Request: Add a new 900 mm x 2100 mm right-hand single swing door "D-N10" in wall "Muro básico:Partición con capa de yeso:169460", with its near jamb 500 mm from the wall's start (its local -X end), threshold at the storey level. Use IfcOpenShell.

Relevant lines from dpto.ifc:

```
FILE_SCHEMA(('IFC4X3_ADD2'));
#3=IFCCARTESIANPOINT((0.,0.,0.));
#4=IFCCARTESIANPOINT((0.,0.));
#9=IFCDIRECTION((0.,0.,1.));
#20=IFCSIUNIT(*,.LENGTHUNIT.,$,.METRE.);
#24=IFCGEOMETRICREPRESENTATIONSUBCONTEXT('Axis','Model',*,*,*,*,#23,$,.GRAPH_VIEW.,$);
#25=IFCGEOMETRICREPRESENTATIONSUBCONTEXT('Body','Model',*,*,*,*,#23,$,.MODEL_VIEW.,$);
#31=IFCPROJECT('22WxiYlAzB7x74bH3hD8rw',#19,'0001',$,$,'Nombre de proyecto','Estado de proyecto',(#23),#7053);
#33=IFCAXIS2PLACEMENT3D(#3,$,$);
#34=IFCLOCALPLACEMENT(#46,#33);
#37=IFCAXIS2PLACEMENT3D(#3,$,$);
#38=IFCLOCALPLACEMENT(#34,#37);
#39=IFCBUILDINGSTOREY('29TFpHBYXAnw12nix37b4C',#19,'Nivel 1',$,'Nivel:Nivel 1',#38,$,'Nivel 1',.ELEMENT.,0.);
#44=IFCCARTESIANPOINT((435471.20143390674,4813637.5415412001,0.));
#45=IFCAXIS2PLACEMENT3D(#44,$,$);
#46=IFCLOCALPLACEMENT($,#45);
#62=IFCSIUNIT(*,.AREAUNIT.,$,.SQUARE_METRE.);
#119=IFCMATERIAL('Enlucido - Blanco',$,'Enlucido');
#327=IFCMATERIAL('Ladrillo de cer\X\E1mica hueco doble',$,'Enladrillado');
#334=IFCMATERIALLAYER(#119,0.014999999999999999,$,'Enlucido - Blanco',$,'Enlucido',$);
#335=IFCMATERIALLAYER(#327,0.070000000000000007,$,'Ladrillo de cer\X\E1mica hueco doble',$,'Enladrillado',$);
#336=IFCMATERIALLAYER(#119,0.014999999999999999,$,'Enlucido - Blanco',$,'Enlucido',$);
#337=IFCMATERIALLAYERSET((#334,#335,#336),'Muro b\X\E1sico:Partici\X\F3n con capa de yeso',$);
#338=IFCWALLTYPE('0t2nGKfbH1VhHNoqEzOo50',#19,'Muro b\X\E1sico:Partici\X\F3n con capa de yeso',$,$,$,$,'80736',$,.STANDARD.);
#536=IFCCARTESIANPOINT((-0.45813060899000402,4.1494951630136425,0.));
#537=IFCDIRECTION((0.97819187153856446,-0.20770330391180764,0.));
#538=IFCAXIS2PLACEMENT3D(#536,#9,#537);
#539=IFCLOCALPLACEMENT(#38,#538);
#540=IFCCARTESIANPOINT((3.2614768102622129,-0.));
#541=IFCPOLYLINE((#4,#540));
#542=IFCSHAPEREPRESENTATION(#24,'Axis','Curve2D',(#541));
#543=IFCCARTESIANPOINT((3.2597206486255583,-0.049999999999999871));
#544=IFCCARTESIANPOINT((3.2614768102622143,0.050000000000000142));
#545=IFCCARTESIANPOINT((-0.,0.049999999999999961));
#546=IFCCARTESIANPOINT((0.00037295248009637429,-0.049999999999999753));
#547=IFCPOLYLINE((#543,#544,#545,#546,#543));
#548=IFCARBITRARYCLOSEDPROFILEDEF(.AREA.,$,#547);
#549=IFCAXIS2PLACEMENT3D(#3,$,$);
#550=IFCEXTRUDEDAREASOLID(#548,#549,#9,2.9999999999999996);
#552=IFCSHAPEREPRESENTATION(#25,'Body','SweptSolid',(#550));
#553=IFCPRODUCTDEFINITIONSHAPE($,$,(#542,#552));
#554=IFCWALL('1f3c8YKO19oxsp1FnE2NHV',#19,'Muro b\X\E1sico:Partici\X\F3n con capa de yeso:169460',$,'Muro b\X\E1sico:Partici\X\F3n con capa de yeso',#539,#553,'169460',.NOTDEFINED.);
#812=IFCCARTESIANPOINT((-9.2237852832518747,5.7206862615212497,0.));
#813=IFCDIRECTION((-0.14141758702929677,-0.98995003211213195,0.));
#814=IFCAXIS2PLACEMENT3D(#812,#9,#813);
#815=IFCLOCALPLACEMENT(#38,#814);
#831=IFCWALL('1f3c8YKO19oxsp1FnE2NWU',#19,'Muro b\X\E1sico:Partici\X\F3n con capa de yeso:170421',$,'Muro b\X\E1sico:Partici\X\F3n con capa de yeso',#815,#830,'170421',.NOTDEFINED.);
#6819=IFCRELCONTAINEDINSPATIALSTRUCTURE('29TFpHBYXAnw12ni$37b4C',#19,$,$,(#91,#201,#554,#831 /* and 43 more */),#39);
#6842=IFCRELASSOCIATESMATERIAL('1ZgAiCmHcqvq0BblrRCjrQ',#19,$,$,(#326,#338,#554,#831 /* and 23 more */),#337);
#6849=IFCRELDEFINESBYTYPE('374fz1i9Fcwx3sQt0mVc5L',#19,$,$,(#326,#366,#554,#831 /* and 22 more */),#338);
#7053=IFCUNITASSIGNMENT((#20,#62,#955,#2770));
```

```python
import numpy as np
import ifcopenshell
import ifcopenshell.api.feature
import ifcopenshell.api.geometry
import ifcopenshell.api.root
import ifcopenshell.api.spatial
import ifcopenshell.geom
import ifcopenshell.util.element
import ifcopenshell.util.placement
import ifcopenshell.util.representation
import ifcopenshell.util.shape
import ifcopenshell.util.unit

model = ifcopenshell.open("dpto.ifc")
unit_scale = ifcopenshell.util.unit.calculate_unit_scale(model)
settings = ifcopenshell.geom.settings()


def volume(element):
    """Net volume in cubic metres, openings subtracted."""
    shape = ifcopenshell.geom.create_shape(settings, element)
    return ifcopenshell.util.shape.get_volume(shape.geometry)


wall = model.by_guid("1f3c8YKO19oxsp1FnE2NHV")
storey = ifcopenshell.util.element.get_container(wall, ifc_class="IfcBuildingStorey")
context = ifcopenshell.util.representation.get_context(model, "Model", "Body", "MODEL_VIEW")
before = volume(wall)

width, height, from_end, sill = 0.9, 2.1, 0.5, 0.0  # metres

# The wall runs along its own X axis, and the end named is its -X end.
wall_shape = ifcopenshell.geom.create_shape(settings, wall)
x, y, z = ifcopenshell.util.shape.get_vertices(wall_shape.geometry).T
start = x.min() + from_end
face, thickness = float(y.min()), float(y.max() - y.min())
wall_matrix = ifcopenshell.util.placement.get_local_placement(wall.ObjectPlacement)
level = ifcopenshell.util.placement.get_local_placement(storey.ObjectPlacement)[2, 3]


def in_wall(x, y):
    """Placement at x, y metres in the wall's axes, at sill height."""
    matrix = wall_matrix.copy()
    matrix[:, 3] = wall_matrix @ np.array([x / unit_scale, y / unit_scale, 0.0, 1.0])
    matrix[2, 3] = level + sill / unit_scale
    return matrix


# Opening: a box that overshoots both wall faces by 50 mm.
opening = ifcopenshell.api.root.create_entity(model, ifc_class="IfcOpeningElement", predefined_type="OPENING")
box = ifcopenshell.api.geometry.add_wall_representation(
    model, context=context, length=width, height=height, thickness=thickness + 0.1
)
ifcopenshell.api.geometry.assign_representation(model, product=opening, representation=box)
ifcopenshell.api.geometry.edit_object_placement(model, product=opening, matrix=in_wall(start, face - 0.05), is_si=False)
ifcopenshell.api.feature.add_feature(model, feature=opening, element=wall)

door = ifcopenshell.api.root.create_entity(model, ifc_class="IfcDoor", name="D-N10", predefined_type="DOOR")
door.OverallWidth, door.OverallHeight = width / unit_scale, height / unit_scale
door.OperationType = "SINGLE_SWING_RIGHT"
body = ifcopenshell.api.geometry.add_door_representation(
    model,
    context=context,
    overall_width=door.OverallWidth,
    overall_height=door.OverallHeight,
    operation_type="SINGLE_SWING_RIGHT",
    lining_properties={"LiningDepth": thickness / unit_scale, "ThresholdDepth": thickness / unit_scale},
)
ifcopenshell.api.geometry.assign_representation(model, product=door, representation=body)
ifcopenshell.api.spatial.assign_container(model, products=[door], relating_structure=storey)
ifcopenshell.api.feature.add_filling(model, opening=opening, element=door)

# The lining spans the wall, so the door starts at the wall face.
ifcopenshell.api.geometry.edit_object_placement(model, product=door, matrix=in_wall(start, face), is_si=False)

after = volume(wall)

print(f"wall volume {before:.3f} -> {after:.3f} m3")

model.write("dpto_rev.ifc")
```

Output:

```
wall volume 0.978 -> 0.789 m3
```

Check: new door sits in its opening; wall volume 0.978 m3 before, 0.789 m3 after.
